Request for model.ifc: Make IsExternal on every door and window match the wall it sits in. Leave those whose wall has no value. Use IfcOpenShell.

First a look at what the model holds.

```python
import ifcopenshell
import ifcopenshell.util.element

model = ifcopenshell.open("model.ifc")
print(model.schema)
seen = {}
for e in model.by_type("IfcDoor") + model.by_type("IfcWindow"):
    if not e.FillsVoids:
        continue
    host = e.FillsVoids[0].RelatingOpeningElement.VoidsElements[0].RelatingBuildingElement
    own = ifcopenshell.util.element.get_pset(e, f"Pset_{e.is_a()[3:].removesuffix('StandardCase')}Common", "IsExternal")
    wall = ifcopenshell.util.element.get_pset(host, "Pset_WallCommon", "IsExternal")
    seen[e.is_a(), own, wall] = seen.get((e.is_a(), own, wall), 0) + 1
for (cls, own, wall), count in sorted(seen.items(), key=str):
    print(count, cls, "IsExternal:", own, "| host wall:", wall)
```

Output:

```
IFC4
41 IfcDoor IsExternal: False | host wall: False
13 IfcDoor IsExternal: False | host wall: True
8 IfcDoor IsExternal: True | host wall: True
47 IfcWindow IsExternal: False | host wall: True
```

```python
import ifcopenshell
import ifcopenshell.api.pset
import ifcopenshell.util.element

model = ifcopenshell.open("model.ifc")

count = 0
for ifc_class, pset_name in (("IfcDoor", "Pset_DoorCommon"), ("IfcWindow", "Pset_WindowCommon")):
    for e in model.by_type(ifc_class):
        if not e.FillsVoids:
            continue
        host = e.FillsVoids[0].RelatingOpeningElement.VoidsElements[0].RelatingBuildingElement
        external = ifcopenshell.util.element.get_pset(host, "Pset_WallCommon", "IsExternal")
        if external is None or ifcopenshell.util.element.get_pset(e, pset_name, "IsExternal") == external:
            continue
        pset = ifcopenshell.api.pset.add_pset(model, product=e, name=pset_name)
        ifcopenshell.api.pset.edit_pset(model, pset=pset, properties={"IsExternal": external})
        count += 1

print(count, "updated")

model.write("model_v2.ifc")
```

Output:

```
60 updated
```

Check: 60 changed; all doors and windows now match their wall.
